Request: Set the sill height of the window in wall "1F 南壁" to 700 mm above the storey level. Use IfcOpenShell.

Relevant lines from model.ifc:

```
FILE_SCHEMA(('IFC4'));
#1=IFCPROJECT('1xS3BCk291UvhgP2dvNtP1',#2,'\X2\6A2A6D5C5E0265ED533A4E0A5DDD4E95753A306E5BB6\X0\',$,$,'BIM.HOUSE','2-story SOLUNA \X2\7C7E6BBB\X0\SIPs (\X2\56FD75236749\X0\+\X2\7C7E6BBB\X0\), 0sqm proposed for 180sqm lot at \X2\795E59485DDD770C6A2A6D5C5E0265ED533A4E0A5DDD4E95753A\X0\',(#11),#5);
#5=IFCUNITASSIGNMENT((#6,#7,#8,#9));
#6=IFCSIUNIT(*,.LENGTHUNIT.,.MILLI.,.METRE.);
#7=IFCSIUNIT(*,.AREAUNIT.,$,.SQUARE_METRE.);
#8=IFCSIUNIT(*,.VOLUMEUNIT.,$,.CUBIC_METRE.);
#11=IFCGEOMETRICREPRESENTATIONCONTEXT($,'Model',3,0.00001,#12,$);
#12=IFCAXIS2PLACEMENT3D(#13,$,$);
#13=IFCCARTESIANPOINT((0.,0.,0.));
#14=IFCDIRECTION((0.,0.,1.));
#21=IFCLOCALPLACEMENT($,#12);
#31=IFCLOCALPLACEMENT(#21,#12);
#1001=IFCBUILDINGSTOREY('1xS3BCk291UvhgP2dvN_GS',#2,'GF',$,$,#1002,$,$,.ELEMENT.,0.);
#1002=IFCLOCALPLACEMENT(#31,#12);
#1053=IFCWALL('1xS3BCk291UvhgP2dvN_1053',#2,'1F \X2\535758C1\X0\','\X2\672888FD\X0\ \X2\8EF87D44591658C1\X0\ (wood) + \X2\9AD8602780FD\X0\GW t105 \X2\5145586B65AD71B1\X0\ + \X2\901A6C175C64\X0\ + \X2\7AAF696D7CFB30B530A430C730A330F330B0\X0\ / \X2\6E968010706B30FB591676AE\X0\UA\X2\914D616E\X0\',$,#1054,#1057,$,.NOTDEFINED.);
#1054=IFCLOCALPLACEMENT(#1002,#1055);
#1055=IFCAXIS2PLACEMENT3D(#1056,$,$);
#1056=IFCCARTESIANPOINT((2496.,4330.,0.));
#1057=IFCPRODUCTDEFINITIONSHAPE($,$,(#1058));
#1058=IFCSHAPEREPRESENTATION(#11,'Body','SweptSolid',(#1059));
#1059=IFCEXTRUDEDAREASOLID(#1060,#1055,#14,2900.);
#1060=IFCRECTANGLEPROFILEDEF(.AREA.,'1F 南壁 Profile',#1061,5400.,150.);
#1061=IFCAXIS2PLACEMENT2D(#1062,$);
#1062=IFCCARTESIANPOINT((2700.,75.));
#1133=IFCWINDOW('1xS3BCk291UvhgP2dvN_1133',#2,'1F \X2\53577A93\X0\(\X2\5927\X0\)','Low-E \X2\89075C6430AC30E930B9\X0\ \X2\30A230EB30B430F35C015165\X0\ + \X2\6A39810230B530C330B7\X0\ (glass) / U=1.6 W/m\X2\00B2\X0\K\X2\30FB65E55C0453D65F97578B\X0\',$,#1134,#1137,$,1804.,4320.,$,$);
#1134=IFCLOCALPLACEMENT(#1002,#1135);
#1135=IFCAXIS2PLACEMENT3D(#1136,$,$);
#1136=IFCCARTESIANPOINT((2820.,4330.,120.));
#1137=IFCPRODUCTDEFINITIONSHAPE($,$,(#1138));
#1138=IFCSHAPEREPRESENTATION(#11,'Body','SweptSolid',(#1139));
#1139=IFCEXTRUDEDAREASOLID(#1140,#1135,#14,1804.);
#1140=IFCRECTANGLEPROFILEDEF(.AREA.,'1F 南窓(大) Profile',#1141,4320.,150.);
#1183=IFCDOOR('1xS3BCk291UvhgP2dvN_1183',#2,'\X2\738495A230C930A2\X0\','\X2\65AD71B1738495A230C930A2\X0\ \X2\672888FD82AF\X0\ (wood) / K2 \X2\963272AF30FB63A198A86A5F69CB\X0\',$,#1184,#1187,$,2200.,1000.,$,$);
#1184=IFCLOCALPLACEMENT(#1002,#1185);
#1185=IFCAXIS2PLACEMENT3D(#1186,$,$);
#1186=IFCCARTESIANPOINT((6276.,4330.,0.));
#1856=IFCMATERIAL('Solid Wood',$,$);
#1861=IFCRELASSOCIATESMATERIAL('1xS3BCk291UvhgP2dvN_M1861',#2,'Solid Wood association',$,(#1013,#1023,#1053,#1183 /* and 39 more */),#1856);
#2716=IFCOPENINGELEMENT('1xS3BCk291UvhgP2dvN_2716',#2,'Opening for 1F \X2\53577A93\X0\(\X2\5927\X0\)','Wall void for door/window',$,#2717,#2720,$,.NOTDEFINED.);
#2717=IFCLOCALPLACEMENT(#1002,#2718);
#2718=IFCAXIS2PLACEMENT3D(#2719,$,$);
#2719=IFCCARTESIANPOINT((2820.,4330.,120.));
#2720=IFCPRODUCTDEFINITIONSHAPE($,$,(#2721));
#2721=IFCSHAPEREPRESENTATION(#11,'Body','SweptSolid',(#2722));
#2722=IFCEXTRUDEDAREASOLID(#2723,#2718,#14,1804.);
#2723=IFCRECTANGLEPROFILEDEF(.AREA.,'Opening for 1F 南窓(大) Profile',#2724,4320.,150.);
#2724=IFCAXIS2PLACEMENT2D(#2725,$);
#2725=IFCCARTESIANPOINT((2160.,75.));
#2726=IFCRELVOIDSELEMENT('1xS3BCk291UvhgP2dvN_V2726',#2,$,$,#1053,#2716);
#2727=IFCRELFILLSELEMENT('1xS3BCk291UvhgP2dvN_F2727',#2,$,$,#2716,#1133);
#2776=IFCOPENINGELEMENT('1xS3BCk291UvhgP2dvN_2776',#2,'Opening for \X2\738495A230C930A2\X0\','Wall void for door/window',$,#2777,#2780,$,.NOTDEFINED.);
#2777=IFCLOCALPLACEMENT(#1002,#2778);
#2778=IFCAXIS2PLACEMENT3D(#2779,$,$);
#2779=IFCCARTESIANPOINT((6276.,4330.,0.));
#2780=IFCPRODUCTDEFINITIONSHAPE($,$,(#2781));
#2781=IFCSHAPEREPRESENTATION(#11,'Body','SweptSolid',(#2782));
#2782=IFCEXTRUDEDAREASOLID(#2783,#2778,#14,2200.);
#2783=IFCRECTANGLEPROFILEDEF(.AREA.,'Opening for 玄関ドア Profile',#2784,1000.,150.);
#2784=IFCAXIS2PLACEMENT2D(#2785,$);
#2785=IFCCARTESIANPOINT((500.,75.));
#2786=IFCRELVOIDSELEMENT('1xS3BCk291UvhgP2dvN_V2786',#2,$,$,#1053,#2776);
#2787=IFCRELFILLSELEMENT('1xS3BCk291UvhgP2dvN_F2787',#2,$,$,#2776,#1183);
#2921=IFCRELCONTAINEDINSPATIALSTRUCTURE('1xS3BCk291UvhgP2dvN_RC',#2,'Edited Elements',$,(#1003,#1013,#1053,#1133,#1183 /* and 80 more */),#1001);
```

```python
import numpy as np
import ifcopenshell
import ifcopenshell.api.geometry
import ifcopenshell.geom
import ifcopenshell.util.element
import ifcopenshell.util.placement
import ifcopenshell.util.shape
import ifcopenshell.util.unit

model = ifcopenshell.open("model.ifc")
unit_scale = ifcopenshell.util.unit.calculate_unit_scale(model)

window = model.by_id(1133)
opening = window.FillsVoids[0].RelatingOpeningElement
storey = ifcopenshell.util.element.get_container(window, ifc_class="IfcBuildingStorey")
level = ifcopenshell.util.placement.get_local_placement(storey.ObjectPlacement)[2, 3]

# The opening's origin need not be at the sill, so measure its lowest point.
shape = ifcopenshell.geom.create_shape(ifcopenshell.geom.settings(), opening)
bottom = ifcopenshell.util.shape.get_shape_bottom_elevation(shape, shape.geometry) / unit_scale
dz = level + 0.7 / unit_scale - bottom

shift = np.array([0.0, 0.0, dz])
# The window is not placed relative to its opening, so move both.
for product in (opening, window):
    matrix = ifcopenshell.util.placement.get_local_placement(product.ObjectPlacement)
    matrix[:3, 3] += shift
    ifcopenshell.api.geometry.edit_object_placement(model, product=product, matrix=matrix, is_si=False)

print(f"moved by {dz * unit_scale:+.3f} m")

model.write("model_v2.ifc")
```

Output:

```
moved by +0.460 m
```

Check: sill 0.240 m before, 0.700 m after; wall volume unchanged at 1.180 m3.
